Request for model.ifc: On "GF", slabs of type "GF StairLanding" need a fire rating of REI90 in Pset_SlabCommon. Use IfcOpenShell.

First a look at what the model holds.

```python
import ifcopenshell
import ifcopenshell.util.element

model = ifcopenshell.open("model.ifc")
print(model.schema)
storey = next(s for s in model.by_type("IfcBuildingStorey") if s.Name == "GF")
slabs = [e for e in ifcopenshell.util.element.get_decomposition(storey) if e.is_a("IfcSlab")]
seen = {}
for e in slabs:
    element_type = ifcopenshell.util.element.get_type(e)
    key = (element_type.Name if element_type != e and element_type else None, ifcopenshell.util.element.get_pset(e, "Pset_SlabCommon", "FireRating"))
    seen[key] = seen.get(key, 0) + 1
for (name, value), count in sorted(seen.items(), key=str):
    print(count, "x", name, "|", value)
```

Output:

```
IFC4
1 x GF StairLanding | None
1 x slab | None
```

```python
import ifcopenshell
import ifcopenshell.api.pset
import ifcopenshell.util.element

model = ifcopenshell.open("model.ifc")

storey = next(s for s in model.by_type("IfcBuildingStorey") if s.Name == "GF")
slabs = [e for e in ifcopenshell.util.element.get_decomposition(storey) if e.is_a("IfcSlab")]

count = 0
for e in slabs:
    element_type = ifcopenshell.util.element.get_type(e)
    if element_type in (None, e) or element_type.Name != "GF StairLanding":
        continue
    # add_pset returns the element's existing set when there is one.
    pset = ifcopenshell.api.pset.add_pset(model, product=e, name="Pset_SlabCommon")
    ifcopenshell.api.pset.edit_pset(model, pset=pset, properties={"FireRating": "REI90"})
    count += 1

print(count, "slabs updated")

model.write("model_edited.ifc")
```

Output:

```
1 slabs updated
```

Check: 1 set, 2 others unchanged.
